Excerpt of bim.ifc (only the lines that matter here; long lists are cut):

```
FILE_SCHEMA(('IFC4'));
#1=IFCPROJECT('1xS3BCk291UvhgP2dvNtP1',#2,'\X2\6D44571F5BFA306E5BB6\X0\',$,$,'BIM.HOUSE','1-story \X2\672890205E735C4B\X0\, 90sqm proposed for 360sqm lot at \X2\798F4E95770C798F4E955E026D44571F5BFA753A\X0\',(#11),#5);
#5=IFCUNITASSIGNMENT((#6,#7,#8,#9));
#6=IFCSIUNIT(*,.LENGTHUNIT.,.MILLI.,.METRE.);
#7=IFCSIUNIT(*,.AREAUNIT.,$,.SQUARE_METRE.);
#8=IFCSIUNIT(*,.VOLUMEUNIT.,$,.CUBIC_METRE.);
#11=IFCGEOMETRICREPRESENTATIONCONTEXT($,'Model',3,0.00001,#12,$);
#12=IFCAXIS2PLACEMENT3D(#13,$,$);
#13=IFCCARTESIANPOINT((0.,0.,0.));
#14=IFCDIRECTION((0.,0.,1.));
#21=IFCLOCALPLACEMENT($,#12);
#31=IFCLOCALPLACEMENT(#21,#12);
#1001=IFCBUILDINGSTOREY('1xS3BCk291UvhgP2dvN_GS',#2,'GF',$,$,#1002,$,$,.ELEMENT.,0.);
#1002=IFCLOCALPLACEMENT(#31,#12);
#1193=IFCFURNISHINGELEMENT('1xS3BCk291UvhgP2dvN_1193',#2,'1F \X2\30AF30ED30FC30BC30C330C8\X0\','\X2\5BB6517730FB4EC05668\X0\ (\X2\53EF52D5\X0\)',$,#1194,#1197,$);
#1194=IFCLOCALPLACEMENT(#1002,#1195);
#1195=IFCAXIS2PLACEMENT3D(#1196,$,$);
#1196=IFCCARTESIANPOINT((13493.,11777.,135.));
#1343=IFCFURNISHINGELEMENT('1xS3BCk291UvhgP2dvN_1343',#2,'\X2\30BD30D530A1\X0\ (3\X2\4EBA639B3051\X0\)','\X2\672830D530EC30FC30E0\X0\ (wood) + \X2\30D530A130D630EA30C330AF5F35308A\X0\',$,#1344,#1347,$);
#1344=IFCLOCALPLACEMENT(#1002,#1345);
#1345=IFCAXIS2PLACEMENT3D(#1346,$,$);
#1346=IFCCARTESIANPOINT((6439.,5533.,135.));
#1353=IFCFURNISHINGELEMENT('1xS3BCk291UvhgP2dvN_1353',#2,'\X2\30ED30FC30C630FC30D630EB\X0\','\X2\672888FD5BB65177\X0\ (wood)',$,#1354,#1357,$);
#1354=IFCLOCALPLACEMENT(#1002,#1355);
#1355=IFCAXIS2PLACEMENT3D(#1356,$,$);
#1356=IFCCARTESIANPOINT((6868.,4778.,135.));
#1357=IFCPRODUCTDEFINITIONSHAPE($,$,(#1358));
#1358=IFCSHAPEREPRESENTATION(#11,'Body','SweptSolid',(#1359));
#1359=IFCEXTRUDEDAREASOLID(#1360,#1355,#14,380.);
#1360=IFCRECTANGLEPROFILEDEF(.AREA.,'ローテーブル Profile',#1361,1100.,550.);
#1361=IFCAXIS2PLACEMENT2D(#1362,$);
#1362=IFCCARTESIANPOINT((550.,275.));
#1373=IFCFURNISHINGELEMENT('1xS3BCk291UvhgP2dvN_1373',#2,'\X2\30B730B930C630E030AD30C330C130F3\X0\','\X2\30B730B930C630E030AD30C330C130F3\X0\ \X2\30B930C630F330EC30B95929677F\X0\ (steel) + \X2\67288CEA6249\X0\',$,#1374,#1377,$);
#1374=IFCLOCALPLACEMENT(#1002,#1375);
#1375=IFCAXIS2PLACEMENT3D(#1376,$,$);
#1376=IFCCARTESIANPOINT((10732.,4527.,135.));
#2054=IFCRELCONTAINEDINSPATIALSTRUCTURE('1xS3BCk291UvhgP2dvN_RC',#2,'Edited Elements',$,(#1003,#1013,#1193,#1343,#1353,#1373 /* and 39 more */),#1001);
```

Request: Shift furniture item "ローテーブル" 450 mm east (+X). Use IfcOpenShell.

```python
import ifcopenshell
import ifcopenshell.api.geometry
import ifcopenshell.util.placement
import ifcopenshell.util.unit

model = ifcopenshell.open("bim.ifc")
unit_scale = ifcopenshell.util.unit.calculate_unit_scale(model)

item = model.by_id(1353)
matrix = ifcopenshell.util.placement.get_local_placement(item.ObjectPlacement)
matrix[0, 3] += 0.45 / unit_scale
ifcopenshell.api.geometry.edit_object_placement(model, product=item, matrix=matrix, is_si=False)

print(ifcopenshell.util.placement.get_local_placement(item.ObjectPlacement).round(3) + 0.0)

model.write("bim_v2.ifc")
```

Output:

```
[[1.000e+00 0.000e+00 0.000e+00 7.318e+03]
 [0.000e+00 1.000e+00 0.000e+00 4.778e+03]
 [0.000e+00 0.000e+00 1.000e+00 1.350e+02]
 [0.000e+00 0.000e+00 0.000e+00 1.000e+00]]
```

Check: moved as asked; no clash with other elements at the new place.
